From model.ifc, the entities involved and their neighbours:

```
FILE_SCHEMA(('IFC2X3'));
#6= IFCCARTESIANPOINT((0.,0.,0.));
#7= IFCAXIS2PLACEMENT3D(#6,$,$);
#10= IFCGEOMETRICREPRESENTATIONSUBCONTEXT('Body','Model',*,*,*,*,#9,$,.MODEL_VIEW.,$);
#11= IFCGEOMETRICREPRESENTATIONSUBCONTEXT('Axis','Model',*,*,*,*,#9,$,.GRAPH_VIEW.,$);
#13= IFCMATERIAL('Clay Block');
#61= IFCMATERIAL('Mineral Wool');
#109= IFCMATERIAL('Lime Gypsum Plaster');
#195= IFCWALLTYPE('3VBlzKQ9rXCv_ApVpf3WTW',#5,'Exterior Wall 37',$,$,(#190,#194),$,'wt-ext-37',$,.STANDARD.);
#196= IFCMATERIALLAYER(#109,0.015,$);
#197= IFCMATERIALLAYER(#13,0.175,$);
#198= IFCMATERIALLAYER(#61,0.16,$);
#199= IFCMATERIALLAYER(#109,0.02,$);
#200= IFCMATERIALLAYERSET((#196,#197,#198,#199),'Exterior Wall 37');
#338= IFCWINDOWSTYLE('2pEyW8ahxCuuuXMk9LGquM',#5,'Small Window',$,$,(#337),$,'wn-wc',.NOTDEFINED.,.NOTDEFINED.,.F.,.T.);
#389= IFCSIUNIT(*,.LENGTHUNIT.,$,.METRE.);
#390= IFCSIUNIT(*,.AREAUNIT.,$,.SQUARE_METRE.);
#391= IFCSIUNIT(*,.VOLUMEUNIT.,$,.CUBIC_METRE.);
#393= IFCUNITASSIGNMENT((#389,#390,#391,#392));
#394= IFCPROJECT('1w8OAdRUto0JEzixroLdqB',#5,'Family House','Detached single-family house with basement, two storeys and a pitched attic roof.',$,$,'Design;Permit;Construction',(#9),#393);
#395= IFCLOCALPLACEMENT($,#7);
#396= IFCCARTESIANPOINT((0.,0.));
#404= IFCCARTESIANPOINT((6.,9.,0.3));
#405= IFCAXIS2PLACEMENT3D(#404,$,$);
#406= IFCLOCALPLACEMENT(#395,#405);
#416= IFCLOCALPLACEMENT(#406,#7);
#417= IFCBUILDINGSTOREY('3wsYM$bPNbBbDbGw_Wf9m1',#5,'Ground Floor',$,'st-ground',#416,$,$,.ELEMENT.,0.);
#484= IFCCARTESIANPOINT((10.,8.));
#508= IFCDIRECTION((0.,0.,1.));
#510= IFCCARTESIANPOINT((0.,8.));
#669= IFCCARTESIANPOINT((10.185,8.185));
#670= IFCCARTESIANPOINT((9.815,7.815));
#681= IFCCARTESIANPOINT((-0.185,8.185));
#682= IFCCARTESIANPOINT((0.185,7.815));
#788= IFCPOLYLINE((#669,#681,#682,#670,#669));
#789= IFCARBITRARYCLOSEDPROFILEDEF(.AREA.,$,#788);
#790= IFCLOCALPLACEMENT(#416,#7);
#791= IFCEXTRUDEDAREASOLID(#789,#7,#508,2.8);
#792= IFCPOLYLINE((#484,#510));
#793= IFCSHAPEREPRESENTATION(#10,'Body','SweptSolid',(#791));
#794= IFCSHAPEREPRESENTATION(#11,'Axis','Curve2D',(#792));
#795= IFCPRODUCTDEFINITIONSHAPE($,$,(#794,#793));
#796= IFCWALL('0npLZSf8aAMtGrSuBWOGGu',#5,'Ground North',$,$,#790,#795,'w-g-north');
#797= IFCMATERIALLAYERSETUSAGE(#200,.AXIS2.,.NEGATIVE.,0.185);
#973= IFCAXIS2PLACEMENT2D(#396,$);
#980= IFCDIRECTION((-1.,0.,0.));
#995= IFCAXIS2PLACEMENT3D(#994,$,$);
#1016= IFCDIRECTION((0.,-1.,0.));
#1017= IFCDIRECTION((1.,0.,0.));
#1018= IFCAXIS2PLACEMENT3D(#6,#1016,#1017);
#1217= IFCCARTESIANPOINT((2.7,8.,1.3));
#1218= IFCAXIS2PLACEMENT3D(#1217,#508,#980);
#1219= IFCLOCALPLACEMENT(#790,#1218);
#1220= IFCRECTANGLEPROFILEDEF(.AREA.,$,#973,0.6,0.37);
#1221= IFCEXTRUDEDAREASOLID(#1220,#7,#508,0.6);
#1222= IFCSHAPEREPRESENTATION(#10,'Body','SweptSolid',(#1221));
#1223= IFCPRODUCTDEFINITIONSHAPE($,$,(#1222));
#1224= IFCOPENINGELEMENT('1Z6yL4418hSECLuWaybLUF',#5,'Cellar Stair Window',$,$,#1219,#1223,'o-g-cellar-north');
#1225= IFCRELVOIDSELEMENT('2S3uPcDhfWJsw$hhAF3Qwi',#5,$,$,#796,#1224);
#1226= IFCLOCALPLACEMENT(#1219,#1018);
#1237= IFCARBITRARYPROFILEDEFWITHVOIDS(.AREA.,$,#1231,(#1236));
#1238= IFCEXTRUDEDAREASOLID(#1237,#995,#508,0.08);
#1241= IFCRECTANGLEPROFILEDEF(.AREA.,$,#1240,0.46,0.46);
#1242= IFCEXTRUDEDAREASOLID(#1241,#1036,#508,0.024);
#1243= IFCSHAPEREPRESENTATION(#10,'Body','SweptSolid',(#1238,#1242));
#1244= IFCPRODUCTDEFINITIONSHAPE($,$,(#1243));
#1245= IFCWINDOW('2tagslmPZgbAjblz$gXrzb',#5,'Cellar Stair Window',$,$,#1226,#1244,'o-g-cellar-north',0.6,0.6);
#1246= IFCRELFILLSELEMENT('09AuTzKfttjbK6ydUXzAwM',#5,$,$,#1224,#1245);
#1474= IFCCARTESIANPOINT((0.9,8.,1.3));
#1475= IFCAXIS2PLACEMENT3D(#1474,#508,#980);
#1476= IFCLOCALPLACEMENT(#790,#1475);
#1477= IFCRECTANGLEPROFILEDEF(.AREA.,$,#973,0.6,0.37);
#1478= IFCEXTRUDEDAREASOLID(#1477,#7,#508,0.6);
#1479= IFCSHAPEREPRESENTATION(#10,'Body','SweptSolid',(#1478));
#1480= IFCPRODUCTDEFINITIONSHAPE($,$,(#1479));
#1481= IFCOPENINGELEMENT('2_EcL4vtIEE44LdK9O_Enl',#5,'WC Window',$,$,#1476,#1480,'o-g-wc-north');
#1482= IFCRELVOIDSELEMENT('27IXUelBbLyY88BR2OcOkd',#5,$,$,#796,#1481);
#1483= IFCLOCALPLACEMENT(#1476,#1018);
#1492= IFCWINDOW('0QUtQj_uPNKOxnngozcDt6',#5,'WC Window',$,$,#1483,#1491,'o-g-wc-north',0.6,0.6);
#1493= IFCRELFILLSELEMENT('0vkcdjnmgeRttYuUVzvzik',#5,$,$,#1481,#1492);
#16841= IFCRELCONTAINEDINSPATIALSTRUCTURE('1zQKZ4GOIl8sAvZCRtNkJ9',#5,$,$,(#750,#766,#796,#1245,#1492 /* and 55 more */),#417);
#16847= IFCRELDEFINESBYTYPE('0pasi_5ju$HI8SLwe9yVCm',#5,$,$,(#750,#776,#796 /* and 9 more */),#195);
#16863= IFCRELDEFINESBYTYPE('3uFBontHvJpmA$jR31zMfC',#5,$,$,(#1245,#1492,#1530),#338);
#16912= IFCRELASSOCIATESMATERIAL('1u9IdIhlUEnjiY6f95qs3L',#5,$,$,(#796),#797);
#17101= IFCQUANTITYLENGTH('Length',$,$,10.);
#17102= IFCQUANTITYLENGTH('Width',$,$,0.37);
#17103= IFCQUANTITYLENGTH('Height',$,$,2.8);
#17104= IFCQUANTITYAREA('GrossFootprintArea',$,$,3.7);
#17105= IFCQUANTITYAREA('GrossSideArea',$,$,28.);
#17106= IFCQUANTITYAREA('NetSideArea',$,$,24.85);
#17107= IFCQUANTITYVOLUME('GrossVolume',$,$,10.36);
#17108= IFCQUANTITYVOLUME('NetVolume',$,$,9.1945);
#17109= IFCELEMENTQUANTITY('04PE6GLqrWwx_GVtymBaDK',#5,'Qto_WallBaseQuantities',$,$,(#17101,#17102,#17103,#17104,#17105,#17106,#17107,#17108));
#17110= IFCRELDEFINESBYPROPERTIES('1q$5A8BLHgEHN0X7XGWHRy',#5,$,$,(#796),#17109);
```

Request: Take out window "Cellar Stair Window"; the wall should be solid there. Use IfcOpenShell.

```python
import ifcopenshell
import ifcopenshell.api.feature
import ifcopenshell.api.pset
import ifcopenshell.api.root
import ifcopenshell.geom
import ifcopenshell.util.element
import ifcopenshell.util.shape
import ifcopenshell.util.unit

model = ifcopenshell.open("model.ifc")
area_scale = ifcopenshell.util.unit.calculate_unit_scale(model, "AREAUNIT")
volume_scale = ifcopenshell.util.unit.calculate_unit_scale(model, "VOLUMEUNIT")
settings = ifcopenshell.geom.settings()


def volume(element):
    """Net volume in cubic metres, openings subtracted."""
    shape = ifcopenshell.geom.create_shape(settings, element)
    return ifcopenshell.util.shape.get_volume(shape.geometry)


window = model.by_guid("2tagslmPZgbAjblz$gXrzb")
opening = window.FillsVoids[0].RelatingOpeningElement
wall = opening.VoidsElements[0].RelatingBuildingElement
before = volume(wall)

ifcopenshell.api.root.remove_product(model, product=window)
ifcopenshell.api.feature.remove_feature(model, feature=opening)

after = volume(wall)
thickness = 0.37  # wall thickness in metres

# Update the wall's stored quantities.
qto = model.by_id(ifcopenshell.util.element.get_pset(wall, "Qto_WallBaseQuantities", should_inherit=False)["id"])
ifcopenshell.api.pset.edit_qto(model, qto=qto, properties={
    "NetSideArea": after / thickness / area_scale,
    "NetVolume": after / volume_scale,
})

print(f"wall volume {before:.3f} -> {after:.3f} m3")

model.write("model_v2.ifc")
```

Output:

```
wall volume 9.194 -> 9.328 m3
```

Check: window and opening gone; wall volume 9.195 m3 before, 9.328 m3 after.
